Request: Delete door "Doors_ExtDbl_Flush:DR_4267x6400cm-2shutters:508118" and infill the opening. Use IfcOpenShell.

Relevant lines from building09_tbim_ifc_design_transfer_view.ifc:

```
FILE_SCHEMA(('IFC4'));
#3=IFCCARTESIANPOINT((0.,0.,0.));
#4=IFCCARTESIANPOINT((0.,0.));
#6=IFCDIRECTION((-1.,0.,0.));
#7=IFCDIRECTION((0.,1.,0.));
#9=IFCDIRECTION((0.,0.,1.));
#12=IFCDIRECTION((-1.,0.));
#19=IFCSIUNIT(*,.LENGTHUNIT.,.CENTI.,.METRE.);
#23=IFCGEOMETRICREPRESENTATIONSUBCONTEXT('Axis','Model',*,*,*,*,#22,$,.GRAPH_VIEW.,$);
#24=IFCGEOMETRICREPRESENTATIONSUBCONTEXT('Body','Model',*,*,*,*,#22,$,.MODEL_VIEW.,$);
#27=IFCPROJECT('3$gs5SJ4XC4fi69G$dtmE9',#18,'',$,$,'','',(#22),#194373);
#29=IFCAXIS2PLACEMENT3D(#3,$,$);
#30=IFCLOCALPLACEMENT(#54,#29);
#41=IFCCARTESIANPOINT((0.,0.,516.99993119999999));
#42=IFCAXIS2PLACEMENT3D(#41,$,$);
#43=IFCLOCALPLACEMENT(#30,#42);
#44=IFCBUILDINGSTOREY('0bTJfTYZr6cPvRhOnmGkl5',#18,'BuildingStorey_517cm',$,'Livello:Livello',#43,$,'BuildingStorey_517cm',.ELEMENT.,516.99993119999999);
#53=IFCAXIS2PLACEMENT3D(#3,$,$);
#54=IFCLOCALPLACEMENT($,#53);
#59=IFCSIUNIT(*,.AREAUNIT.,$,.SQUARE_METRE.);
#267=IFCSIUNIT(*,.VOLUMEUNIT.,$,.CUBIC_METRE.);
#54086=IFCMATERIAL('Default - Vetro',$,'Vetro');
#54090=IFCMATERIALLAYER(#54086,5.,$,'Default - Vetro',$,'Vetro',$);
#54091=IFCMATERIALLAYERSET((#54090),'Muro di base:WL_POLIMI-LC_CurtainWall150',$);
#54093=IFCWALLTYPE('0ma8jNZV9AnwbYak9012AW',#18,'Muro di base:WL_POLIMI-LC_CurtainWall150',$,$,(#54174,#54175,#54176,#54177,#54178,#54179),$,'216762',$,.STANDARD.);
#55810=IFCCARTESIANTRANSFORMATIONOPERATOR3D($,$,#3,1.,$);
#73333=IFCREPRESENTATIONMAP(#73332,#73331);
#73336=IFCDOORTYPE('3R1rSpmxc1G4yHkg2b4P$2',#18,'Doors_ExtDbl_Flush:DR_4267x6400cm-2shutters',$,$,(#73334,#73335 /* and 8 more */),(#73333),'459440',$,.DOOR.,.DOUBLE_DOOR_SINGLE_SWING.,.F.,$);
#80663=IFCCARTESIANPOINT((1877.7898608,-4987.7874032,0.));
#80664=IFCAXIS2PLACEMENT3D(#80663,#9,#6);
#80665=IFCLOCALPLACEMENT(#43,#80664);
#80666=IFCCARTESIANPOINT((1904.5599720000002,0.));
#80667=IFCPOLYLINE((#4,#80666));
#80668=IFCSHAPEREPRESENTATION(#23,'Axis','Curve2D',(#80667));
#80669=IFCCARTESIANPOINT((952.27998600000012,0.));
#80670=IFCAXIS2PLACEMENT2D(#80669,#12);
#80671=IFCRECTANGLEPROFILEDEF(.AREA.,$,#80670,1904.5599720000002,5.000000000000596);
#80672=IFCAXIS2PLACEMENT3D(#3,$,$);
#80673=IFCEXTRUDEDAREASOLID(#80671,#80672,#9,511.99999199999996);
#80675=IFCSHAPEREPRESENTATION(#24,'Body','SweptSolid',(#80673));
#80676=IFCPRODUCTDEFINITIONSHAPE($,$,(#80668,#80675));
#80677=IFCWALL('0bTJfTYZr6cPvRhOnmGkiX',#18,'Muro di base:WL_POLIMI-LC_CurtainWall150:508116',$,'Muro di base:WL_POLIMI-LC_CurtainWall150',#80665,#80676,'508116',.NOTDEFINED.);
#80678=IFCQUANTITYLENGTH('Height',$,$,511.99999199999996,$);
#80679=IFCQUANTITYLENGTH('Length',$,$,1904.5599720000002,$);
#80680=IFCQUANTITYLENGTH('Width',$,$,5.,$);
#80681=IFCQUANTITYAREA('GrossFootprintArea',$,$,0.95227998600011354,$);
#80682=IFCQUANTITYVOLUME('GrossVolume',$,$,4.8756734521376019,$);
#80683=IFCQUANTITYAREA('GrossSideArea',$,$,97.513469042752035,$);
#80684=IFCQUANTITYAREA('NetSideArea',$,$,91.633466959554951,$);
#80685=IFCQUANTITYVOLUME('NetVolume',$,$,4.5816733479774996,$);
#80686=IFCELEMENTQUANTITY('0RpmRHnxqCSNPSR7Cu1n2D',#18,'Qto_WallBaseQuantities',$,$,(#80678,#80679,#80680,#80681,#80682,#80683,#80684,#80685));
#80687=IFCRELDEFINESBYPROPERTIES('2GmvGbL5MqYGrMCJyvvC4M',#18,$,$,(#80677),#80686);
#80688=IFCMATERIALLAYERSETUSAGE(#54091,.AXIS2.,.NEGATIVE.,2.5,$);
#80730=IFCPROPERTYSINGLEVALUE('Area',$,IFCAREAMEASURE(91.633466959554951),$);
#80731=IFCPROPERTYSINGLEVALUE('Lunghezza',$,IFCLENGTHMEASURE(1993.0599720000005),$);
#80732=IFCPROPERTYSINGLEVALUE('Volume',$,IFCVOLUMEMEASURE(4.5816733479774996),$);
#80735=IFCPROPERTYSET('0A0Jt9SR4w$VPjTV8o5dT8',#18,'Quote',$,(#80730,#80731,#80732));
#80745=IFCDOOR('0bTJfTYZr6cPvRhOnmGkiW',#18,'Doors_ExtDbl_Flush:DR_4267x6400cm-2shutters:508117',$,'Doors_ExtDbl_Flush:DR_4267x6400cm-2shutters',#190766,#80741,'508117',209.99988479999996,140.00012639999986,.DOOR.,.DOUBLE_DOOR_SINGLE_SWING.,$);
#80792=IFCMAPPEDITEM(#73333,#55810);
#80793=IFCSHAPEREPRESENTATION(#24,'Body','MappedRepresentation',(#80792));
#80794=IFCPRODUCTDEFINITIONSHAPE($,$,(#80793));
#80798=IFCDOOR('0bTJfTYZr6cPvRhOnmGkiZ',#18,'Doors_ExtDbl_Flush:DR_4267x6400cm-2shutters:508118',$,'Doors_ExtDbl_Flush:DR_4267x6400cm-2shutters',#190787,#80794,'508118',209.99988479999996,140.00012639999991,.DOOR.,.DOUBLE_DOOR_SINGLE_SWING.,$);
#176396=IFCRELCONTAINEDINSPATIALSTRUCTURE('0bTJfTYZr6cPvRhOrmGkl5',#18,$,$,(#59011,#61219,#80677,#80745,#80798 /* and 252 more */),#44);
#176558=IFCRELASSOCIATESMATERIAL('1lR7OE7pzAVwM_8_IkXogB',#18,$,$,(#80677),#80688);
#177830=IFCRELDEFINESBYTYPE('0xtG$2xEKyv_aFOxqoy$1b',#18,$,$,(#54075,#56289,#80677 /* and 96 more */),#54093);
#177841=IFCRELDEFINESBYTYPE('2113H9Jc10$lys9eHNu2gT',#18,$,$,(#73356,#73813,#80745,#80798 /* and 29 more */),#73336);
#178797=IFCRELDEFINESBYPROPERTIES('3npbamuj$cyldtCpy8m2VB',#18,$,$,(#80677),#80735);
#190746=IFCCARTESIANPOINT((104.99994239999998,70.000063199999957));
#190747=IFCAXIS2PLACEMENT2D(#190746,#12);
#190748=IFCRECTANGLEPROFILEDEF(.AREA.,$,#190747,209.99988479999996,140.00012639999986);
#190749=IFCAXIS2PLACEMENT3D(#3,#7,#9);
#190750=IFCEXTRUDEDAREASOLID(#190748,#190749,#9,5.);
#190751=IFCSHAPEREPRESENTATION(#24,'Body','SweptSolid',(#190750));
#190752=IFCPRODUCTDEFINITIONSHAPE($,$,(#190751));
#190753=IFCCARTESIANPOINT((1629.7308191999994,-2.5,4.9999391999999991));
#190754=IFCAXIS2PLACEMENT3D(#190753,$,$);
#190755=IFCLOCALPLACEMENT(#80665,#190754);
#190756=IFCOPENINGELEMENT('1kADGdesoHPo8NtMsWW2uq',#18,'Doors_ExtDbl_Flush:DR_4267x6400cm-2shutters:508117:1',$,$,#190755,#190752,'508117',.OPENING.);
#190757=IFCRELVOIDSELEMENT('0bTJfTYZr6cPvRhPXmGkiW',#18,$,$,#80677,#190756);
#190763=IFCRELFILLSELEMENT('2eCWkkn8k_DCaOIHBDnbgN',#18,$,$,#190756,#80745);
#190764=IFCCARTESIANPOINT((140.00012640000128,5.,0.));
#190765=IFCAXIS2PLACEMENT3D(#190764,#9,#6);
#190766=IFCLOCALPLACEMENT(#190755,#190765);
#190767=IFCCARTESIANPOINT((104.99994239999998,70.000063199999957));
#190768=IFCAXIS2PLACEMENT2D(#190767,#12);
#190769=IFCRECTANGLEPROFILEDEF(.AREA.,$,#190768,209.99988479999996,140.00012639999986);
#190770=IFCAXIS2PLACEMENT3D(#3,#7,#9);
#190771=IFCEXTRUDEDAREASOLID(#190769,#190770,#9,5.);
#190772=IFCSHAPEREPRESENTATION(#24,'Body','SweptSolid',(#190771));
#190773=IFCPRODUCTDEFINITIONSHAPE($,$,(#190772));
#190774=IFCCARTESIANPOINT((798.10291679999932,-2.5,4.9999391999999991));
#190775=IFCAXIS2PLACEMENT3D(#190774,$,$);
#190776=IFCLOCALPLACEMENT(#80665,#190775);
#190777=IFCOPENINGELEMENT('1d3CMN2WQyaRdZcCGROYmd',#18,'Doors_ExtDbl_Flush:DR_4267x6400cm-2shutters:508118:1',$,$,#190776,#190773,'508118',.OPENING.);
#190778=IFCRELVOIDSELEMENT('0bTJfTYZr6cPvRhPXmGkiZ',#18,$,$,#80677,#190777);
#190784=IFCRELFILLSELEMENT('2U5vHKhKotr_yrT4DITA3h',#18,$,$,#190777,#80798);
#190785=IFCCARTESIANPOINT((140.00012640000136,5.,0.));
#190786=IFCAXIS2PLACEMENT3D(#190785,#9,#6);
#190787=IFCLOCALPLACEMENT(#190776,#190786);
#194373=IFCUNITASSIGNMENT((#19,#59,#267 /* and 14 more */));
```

```python
import ifcopenshell
import ifcopenshell.api.feature
import ifcopenshell.api.pset
import ifcopenshell.api.root
import ifcopenshell.geom
import ifcopenshell.util.element
import ifcopenshell.util.shape
import ifcopenshell.util.unit

model = ifcopenshell.open("building09_tbim_ifc_design_transfer_view.ifc")
area_scale = ifcopenshell.util.unit.calculate_unit_scale(model, "AREAUNIT")
volume_scale = ifcopenshell.util.unit.calculate_unit_scale(model, "VOLUMEUNIT")
settings = ifcopenshell.geom.settings()


def volume(element):
    """Net volume in cubic metres, openings subtracted."""
    shape = ifcopenshell.geom.create_shape(settings, element)
    return ifcopenshell.util.shape.get_volume(shape.geometry)


door = model.by_guid("0bTJfTYZr6cPvRhOnmGkiZ")
opening = door.FillsVoids[0].RelatingOpeningElement
wall = opening.VoidsElements[0].RelatingBuildingElement
before = volume(wall)

ifcopenshell.api.root.remove_product(model, product=door)
ifcopenshell.api.feature.remove_feature(model, feature=opening)

after = volume(wall)
thickness = 0.05  # wall thickness in metres

# Update the wall's stored quantities.
qto = model.by_id(ifcopenshell.util.element.get_pset(wall, "Qto_WallBaseQuantities", should_inherit=False)["id"])
ifcopenshell.api.pset.edit_qto(model, qto=qto, properties={
    "NetSideArea": after / thickness / area_scale,
    "NetVolume": after / volume_scale,
})
pset = model.by_id(ifcopenshell.util.element.get_pset(wall, "Quote", should_inherit=False)["id"])
ifcopenshell.api.pset.edit_pset(model, pset=pset, properties={
    "Area": model.create_entity("IfcAreaMeasure", after / thickness / area_scale),
    "Volume": model.create_entity("IfcVolumeMeasure", after / volume_scale),
})

print(f"wall volume {before:.3f} -> {after:.3f} m3")

model.write("building09_tbim_ifc_design_transfer_view-out.ifc")
```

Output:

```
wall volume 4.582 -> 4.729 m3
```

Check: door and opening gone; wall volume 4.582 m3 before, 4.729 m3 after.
